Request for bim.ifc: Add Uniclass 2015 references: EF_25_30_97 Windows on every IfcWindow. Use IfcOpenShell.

First a look at what the model holds.

```python
import ifcopenshell

model = ifcopenshell.open("bim.ifc")
print(model.schema)
print("classifications:", [c.Name for c in model.by_type("IfcClassification")])
for ifc_class in ("IfcDoor", "IfcRoof", "IfcStair", "IfcWall", "IfcWindow"):
    print(ifc_class, len(model.by_type(ifc_class)))
```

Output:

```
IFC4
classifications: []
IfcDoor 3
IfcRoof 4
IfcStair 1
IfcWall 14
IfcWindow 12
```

```python
import ifcopenshell
import ifcopenshell.api.classification

model = ifcopenshell.open("bim.ifc")

system = ifcopenshell.api.classification.add_classification(model, classification="Uniclass 2015")

codes = {
    "IfcWindow": ("EF_25_30_97", "Windows"),
}
for ifc_class, (code, name) in codes.items():
    products = model.by_type(ifc_class)
    ifcopenshell.api.classification.add_reference(
        model, products=products, classification=system, identification=code, name=name
    )
    print(code, len(products))

model.write("bim_v2.ifc")
```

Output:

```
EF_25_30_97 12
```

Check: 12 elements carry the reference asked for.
